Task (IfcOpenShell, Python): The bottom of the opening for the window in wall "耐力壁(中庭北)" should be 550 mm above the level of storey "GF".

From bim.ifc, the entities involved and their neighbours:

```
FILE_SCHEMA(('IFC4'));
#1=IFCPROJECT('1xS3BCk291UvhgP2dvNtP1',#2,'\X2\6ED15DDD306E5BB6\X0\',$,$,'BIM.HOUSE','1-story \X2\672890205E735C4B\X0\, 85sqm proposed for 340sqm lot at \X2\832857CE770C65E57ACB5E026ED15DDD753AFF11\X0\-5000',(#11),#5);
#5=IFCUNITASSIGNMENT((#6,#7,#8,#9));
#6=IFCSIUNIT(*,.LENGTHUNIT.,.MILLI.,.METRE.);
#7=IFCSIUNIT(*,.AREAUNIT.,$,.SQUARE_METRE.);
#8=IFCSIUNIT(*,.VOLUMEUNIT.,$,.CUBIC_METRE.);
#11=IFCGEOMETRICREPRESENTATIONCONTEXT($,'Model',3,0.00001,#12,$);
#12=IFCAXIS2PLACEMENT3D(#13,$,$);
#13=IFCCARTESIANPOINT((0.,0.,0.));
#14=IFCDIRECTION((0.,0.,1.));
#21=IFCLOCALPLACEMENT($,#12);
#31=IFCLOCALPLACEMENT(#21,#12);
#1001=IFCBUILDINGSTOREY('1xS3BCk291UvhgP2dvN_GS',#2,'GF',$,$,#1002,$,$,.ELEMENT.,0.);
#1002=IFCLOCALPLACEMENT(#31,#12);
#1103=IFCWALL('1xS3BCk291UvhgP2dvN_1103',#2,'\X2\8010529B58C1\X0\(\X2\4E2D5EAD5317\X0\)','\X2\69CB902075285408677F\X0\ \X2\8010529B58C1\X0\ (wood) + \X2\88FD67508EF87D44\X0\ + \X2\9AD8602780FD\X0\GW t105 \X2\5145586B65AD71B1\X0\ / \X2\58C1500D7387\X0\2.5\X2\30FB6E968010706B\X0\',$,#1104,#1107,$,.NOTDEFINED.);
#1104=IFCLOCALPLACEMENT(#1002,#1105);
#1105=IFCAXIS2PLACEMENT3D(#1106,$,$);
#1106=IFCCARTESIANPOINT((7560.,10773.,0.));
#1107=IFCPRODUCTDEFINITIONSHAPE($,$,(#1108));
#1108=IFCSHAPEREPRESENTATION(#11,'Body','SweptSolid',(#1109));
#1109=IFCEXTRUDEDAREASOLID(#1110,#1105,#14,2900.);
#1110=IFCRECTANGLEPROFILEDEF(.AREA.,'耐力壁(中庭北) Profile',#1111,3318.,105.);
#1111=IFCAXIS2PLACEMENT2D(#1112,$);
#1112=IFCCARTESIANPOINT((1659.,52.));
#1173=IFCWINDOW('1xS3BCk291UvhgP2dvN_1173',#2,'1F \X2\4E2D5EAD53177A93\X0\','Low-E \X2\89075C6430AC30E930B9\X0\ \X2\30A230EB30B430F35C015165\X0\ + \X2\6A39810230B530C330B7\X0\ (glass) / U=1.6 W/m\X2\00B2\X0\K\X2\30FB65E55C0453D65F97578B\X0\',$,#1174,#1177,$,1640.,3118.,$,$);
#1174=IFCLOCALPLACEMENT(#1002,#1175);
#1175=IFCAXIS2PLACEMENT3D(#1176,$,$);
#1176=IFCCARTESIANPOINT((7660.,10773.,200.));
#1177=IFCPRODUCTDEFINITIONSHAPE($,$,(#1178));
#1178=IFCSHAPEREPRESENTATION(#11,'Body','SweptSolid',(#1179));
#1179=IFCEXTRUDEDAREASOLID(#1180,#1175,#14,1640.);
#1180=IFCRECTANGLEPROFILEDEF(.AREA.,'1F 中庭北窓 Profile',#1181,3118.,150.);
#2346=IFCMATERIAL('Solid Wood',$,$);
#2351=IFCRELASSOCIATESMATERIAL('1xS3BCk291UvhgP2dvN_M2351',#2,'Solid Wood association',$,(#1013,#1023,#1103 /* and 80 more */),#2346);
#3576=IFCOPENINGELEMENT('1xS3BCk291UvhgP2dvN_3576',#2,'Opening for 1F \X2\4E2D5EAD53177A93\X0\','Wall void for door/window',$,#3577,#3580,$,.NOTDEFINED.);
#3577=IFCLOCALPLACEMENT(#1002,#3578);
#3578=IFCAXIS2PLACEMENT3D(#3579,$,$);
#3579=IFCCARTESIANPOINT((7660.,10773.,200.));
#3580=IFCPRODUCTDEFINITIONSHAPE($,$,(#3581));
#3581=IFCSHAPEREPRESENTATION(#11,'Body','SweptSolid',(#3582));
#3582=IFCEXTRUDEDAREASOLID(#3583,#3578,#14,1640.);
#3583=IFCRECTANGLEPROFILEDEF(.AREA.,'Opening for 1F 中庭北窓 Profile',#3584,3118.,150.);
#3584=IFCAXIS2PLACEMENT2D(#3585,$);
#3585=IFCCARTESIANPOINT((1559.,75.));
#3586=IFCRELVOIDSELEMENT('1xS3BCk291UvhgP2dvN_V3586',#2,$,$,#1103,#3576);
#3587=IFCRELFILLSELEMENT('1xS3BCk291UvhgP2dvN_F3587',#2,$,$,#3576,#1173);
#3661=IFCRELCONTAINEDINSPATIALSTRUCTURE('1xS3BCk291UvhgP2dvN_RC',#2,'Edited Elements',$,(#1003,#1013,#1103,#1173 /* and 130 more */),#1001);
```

```python
import numpy as np
import ifcopenshell
import ifcopenshell.api.geometry
import ifcopenshell.geom
import ifcopenshell.util.element
import ifcopenshell.util.placement
import ifcopenshell.util.shape
import ifcopenshell.util.unit

model = ifcopenshell.open("bim.ifc")
unit_scale = ifcopenshell.util.unit.calculate_unit_scale(model)

window = model.by_id(1173)
opening = window.FillsVoids[0].RelatingOpeningElement
storey = ifcopenshell.util.element.get_container(window, ifc_class="IfcBuildingStorey")
level = ifcopenshell.util.placement.get_local_placement(storey.ObjectPlacement)[2, 3]

# The opening's origin need not be at the sill, so measure its lowest point.
shape = ifcopenshell.geom.create_shape(ifcopenshell.geom.settings(), opening)
bottom = ifcopenshell.util.shape.get_shape_bottom_elevation(shape, shape.geometry) / unit_scale
dz = level + 550.0 - bottom

shift = np.array([0.0, 0.0, dz])
# The window is not placed relative to its opening, so move both.
for product in (opening, window):
    matrix = ifcopenshell.util.placement.get_local_placement(product.ObjectPlacement)
    matrix[:3, 3] += shift
    ifcopenshell.api.geometry.edit_object_placement(model, product=product, matrix=matrix, is_si=False)

print(f"moved by {dz * unit_scale:+.3f} m")

model.write("bim_edited.ifc")
```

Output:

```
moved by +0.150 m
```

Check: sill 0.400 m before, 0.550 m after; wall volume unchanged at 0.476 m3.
